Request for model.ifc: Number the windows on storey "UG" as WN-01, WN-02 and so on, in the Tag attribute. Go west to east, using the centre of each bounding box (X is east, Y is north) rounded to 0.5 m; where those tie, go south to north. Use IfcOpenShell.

First a look at what the model holds.

```python
import ifcopenshell
import ifcopenshell.util.element
import ifcopenshell.util.placement

model = ifcopenshell.open("model.ifc")
print(model.schema)
storey = next(s for s in model.by_type("IfcBuildingStorey") if s.Name == "UG")
windows = [e for e in ifcopenshell.util.element.get_decomposition(storey) if e.is_a("IfcWindow")]
for e in sorted(windows, key=lambda e: e.id()):
    origin = ifcopenshell.util.placement.get_local_placement(e.ObjectPlacement)[:3, 3]
    print(e.id(), e.Tag, e.Name, origin.round(2) + 0.0, sep=" | ")
```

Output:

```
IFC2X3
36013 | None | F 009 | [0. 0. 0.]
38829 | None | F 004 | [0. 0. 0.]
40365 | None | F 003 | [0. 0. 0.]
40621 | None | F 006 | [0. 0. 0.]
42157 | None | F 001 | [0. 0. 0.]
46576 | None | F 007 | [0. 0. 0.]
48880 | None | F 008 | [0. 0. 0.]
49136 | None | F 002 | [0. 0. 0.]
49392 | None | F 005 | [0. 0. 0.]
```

```python
import ifcopenshell
import ifcopenshell.geom
import ifcopenshell.util.element
import ifcopenshell.util.shape

model = ifcopenshell.open("model.ifc")
settings = ifcopenshell.geom.settings()
settings.set("use-world-coords", True)


def centre(element):
    shape = ifcopenshell.geom.create_shape(settings, element)
    return ifcopenshell.util.shape.get_bbox_centroid(shape.geometry)


storey = next(s for s in model.by_type("IfcBuildingStorey") if s.Name == "UG")
windows = [e for e in ifcopenshell.util.element.get_decomposition(storey) if e.is_a("IfcWindow")]

# Insertion points can sit at a corner or the storey origin, so sort by the geometry (in metres).
centres = {e: centre(e) for e in windows}
windows.sort(key=lambda e: (round(centres[e][0] / 0.5), centres[e][1]))

for i, e in enumerate(windows, start=1):
    number = f"WN-{i:02d}"
    e.Tag = number
    print(e.id(), number)

model.write("model_rev.ifc")
```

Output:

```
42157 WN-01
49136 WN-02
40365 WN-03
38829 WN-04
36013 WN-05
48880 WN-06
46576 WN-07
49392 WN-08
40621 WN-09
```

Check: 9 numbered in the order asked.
